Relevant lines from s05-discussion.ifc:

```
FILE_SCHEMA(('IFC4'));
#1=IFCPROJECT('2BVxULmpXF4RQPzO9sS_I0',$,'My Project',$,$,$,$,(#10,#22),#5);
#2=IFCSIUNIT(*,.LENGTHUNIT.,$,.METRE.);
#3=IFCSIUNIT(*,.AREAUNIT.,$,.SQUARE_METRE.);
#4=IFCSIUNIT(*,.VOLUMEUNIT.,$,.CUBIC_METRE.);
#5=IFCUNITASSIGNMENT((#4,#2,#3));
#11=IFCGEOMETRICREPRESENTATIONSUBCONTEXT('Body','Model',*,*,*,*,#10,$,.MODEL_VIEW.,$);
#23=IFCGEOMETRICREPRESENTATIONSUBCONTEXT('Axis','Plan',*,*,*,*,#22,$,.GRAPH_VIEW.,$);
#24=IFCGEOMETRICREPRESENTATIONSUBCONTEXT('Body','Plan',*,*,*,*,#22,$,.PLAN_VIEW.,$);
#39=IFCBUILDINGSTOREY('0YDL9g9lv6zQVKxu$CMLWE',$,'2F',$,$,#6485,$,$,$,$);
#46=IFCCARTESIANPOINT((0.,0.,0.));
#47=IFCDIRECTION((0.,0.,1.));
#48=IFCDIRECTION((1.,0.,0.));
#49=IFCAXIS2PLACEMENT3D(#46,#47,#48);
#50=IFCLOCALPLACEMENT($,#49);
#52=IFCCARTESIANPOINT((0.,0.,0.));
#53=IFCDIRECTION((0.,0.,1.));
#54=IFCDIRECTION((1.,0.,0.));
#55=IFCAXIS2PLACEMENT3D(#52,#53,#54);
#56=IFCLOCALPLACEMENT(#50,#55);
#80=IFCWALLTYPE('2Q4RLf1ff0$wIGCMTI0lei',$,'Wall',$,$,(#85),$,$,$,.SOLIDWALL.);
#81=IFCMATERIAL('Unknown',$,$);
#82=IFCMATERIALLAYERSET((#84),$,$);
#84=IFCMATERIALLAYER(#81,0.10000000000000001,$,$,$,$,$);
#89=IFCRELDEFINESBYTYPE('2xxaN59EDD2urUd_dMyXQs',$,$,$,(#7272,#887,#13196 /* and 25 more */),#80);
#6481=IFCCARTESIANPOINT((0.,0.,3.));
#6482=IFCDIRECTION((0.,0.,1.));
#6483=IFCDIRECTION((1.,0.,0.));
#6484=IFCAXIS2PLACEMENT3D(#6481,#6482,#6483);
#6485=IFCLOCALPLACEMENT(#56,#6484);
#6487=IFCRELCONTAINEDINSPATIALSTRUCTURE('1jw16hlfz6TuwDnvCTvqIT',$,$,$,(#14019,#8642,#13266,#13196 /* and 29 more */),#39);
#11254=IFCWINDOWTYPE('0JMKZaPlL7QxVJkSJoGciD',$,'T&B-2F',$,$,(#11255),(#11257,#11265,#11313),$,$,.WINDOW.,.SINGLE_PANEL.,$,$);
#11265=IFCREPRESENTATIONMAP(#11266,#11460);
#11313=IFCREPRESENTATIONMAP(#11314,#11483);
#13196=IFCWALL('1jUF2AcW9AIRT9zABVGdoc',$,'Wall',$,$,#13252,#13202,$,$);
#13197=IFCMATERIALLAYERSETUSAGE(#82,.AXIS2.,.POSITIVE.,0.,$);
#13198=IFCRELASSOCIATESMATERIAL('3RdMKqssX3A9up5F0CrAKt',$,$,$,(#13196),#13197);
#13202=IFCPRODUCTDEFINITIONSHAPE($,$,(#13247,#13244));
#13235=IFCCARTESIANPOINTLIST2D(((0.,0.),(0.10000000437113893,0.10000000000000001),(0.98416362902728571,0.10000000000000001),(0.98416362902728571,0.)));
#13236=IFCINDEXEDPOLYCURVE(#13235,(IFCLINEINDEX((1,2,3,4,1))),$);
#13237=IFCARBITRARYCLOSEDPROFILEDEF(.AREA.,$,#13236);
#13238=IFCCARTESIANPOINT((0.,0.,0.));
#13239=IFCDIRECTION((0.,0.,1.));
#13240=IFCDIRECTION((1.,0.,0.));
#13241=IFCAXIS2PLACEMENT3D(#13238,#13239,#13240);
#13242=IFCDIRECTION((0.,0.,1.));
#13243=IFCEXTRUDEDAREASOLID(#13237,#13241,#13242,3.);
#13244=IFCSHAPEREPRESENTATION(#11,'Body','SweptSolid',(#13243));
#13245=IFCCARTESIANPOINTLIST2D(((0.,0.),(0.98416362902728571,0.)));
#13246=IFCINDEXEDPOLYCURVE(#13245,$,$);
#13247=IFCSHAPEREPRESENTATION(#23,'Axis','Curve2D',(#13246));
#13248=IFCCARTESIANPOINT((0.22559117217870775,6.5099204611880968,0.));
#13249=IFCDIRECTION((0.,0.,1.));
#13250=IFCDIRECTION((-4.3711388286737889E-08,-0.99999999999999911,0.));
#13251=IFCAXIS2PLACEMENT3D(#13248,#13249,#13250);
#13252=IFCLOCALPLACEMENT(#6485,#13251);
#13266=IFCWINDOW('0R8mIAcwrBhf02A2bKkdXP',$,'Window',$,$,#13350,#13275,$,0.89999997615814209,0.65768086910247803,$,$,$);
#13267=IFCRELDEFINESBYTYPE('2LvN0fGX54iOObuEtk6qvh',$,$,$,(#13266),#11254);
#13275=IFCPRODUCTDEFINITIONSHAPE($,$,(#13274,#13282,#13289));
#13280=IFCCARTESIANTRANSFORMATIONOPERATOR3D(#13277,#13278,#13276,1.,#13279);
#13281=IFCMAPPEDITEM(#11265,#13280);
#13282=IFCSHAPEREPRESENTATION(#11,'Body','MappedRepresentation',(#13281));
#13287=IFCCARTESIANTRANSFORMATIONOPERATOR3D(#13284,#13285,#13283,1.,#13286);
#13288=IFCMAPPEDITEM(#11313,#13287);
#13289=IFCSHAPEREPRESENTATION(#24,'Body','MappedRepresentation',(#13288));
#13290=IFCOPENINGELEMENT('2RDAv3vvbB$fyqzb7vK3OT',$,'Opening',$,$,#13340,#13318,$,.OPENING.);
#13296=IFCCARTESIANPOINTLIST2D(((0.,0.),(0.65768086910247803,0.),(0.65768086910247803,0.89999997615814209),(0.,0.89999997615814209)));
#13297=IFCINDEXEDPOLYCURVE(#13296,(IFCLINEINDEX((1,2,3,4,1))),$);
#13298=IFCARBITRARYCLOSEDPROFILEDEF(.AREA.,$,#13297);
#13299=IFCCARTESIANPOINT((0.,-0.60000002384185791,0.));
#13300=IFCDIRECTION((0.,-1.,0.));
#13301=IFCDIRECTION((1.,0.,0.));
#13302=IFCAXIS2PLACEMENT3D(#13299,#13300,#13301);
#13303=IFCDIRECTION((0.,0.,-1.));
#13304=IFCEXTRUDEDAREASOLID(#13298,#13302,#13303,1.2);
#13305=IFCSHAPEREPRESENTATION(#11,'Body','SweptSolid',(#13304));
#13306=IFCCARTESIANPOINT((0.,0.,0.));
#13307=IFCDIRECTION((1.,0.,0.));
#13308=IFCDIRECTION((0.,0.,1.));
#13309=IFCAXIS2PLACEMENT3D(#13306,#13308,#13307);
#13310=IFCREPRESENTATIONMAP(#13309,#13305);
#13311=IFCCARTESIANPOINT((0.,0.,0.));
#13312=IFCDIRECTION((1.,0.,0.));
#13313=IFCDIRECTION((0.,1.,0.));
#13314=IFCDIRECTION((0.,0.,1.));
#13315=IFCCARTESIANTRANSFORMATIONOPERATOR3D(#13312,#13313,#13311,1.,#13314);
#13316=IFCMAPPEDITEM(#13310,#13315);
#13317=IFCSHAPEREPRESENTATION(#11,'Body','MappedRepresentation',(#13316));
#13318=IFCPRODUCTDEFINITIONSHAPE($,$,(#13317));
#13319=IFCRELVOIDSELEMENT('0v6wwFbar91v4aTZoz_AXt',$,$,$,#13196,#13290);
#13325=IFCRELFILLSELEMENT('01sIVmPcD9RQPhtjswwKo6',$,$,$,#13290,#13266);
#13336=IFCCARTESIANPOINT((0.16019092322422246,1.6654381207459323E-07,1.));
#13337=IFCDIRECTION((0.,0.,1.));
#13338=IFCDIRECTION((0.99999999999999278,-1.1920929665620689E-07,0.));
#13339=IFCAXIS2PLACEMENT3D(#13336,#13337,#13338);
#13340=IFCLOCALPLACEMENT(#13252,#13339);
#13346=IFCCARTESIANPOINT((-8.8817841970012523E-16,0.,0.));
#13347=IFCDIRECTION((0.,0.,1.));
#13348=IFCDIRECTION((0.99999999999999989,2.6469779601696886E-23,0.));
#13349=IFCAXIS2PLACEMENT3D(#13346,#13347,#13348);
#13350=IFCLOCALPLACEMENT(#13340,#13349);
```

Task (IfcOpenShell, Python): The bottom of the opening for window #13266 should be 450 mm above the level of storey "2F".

```python
import numpy as np
import ifcopenshell
import ifcopenshell.api.geometry
import ifcopenshell.geom
import ifcopenshell.util.element
import ifcopenshell.util.placement
import ifcopenshell.util.shape
import ifcopenshell.util.unit

model = ifcopenshell.open("s05-discussion.ifc")
unit_scale = ifcopenshell.util.unit.calculate_unit_scale(model)

window = model.by_guid("0R8mIAcwrBhf02A2bKkdXP")
opening = window.FillsVoids[0].RelatingOpeningElement
storey = ifcopenshell.util.element.get_container(window, ifc_class="IfcBuildingStorey")
level = ifcopenshell.util.placement.get_local_placement(storey.ObjectPlacement)[2, 3]

# The opening's origin need not be at the sill, so measure its lowest point.
shape = ifcopenshell.geom.create_shape(ifcopenshell.geom.settings(), opening)
bottom = ifcopenshell.util.shape.get_shape_bottom_elevation(shape, shape.geometry) / unit_scale
dz = level + 0.45 - bottom

shift = np.array([0.0, 0.0, dz])
# The window is placed relative to its opening, so it follows when the opening moves.
matrix = ifcopenshell.util.placement.get_local_placement(opening.ObjectPlacement)
matrix[:3, 3] += shift
ifcopenshell.api.geometry.edit_object_placement(
    model, product=opening, matrix=matrix, is_si=False, should_transform_children=True
)

print(f"moved by {dz * unit_scale:+.3f} m")

model.write("s05-discussion_edited.ifc")
```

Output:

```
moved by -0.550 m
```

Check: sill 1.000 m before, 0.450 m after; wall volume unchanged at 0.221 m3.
